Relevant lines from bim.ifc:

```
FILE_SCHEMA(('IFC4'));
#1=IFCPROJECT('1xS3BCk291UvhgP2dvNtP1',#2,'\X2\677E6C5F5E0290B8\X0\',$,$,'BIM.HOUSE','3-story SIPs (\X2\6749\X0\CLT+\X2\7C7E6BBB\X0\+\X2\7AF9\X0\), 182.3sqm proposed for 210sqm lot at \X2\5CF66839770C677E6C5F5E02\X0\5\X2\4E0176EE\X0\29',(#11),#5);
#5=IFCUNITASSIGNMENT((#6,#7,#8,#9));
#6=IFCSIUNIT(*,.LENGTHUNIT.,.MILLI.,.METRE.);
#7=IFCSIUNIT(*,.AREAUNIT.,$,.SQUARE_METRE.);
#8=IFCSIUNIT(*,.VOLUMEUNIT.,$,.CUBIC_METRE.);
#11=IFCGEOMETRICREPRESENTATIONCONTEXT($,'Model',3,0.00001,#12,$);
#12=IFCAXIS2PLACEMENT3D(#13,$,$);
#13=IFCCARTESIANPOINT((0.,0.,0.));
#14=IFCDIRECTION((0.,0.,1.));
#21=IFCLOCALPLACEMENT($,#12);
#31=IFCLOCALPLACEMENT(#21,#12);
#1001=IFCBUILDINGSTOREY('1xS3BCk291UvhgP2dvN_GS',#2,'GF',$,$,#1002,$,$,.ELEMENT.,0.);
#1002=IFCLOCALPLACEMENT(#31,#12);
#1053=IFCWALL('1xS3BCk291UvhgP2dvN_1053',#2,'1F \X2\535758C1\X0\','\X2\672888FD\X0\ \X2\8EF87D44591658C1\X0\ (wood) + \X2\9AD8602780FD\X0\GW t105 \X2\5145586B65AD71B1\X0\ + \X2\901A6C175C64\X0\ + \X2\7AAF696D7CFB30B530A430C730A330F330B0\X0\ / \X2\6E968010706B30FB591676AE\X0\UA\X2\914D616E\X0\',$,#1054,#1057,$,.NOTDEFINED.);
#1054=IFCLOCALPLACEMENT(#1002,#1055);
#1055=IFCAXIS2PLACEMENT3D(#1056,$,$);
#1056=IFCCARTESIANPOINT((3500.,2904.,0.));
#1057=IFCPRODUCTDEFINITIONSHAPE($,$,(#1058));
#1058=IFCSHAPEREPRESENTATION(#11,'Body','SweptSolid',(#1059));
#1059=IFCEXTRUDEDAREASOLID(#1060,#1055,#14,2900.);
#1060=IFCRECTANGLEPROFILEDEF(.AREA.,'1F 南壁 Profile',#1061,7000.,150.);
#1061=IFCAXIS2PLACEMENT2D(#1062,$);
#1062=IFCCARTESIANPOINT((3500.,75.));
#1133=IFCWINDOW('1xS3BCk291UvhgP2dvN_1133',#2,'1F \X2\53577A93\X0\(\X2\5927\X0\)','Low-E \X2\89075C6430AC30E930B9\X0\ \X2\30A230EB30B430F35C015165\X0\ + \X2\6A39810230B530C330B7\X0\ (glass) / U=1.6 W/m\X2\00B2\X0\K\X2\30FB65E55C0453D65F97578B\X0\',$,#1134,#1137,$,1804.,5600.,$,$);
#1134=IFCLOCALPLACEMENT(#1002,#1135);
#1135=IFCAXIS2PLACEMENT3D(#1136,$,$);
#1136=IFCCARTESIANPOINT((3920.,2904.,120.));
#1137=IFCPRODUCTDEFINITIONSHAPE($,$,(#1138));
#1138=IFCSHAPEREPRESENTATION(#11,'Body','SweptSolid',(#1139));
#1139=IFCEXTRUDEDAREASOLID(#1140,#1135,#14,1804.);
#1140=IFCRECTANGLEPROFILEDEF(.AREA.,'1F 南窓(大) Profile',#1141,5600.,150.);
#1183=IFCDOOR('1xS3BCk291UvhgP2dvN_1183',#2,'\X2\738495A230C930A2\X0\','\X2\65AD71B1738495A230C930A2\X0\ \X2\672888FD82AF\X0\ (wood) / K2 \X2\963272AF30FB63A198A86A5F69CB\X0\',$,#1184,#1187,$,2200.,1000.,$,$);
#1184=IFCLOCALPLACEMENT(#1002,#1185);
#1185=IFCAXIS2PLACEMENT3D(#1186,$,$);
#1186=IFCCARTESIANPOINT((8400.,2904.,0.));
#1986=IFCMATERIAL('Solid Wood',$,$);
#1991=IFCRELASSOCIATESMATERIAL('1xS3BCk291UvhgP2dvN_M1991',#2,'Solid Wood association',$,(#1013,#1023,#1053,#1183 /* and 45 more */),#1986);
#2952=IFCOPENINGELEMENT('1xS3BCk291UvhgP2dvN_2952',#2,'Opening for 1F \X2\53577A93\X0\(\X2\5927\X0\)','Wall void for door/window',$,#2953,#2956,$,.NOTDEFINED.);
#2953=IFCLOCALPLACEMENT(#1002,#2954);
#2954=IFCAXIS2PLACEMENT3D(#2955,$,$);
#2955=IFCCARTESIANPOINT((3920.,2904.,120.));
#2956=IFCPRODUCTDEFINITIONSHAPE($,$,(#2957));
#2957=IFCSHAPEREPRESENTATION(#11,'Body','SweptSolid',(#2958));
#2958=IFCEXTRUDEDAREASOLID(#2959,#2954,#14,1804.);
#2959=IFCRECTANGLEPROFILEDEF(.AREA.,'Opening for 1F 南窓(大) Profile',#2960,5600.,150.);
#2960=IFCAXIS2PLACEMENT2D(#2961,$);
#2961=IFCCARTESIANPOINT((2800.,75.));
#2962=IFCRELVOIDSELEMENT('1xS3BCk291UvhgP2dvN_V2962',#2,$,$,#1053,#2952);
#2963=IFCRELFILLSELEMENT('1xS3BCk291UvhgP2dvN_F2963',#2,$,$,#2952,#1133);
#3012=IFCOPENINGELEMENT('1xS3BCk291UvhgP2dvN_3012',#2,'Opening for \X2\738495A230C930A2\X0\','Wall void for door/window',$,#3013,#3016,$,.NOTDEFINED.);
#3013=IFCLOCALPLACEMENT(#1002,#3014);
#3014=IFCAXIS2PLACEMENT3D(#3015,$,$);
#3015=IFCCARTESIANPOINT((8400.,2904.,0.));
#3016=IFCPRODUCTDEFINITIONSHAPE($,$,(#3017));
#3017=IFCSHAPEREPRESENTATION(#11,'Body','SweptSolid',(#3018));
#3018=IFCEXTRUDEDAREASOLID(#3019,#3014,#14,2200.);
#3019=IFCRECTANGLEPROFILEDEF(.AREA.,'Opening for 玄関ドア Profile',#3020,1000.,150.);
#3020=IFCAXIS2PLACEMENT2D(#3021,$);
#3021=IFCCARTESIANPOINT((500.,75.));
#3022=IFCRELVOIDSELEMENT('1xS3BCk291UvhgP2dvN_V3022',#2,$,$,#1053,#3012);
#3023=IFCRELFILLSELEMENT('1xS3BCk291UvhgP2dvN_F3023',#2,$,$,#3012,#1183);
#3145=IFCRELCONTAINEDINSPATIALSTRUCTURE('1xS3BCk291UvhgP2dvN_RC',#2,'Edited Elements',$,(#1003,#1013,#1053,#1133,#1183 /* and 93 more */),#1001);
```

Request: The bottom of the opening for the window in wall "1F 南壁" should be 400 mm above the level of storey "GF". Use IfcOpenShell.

```python
import numpy as np
import ifcopenshell
import ifcopenshell.api.geometry
import ifcopenshell.geom
import ifcopenshell.util.element
import ifcopenshell.util.placement
import ifcopenshell.util.shape
import ifcopenshell.util.unit

model = ifcopenshell.open("bim.ifc")
unit_scale = ifcopenshell.util.unit.calculate_unit_scale(model)

window = model.by_guid("1xS3BCk291UvhgP2dvN_1133")
opening = window.FillsVoids[0].RelatingOpeningElement
storey = ifcopenshell.util.element.get_container(window, ifc_class="IfcBuildingStorey")
level = ifcopenshell.util.placement.get_local_placement(storey.ObjectPlacement)[2, 3]

# The opening's origin need not be at the sill, so measure its lowest point.
shape = ifcopenshell.geom.create_shape(ifcopenshell.geom.settings(), opening)
bottom = ifcopenshell.util.shape.get_shape_bottom_elevation(shape, shape.geometry) / unit_scale
dz = level + 400.0 - bottom

shift = np.array([0.0, 0.0, dz])
# The window is not placed relative to its opening, so move both.
for product in (opening, window):
    matrix = ifcopenshell.util.placement.get_local_placement(product.ObjectPlacement)
    matrix[:3, 3] += shift
    ifcopenshell.api.geometry.edit_object_placement(model, product=product, matrix=matrix, is_si=False)

print(f"moved by {dz * unit_scale:+.3f} m")

model.write("bim_edited.ifc")
```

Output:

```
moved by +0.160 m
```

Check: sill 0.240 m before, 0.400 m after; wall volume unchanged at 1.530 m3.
